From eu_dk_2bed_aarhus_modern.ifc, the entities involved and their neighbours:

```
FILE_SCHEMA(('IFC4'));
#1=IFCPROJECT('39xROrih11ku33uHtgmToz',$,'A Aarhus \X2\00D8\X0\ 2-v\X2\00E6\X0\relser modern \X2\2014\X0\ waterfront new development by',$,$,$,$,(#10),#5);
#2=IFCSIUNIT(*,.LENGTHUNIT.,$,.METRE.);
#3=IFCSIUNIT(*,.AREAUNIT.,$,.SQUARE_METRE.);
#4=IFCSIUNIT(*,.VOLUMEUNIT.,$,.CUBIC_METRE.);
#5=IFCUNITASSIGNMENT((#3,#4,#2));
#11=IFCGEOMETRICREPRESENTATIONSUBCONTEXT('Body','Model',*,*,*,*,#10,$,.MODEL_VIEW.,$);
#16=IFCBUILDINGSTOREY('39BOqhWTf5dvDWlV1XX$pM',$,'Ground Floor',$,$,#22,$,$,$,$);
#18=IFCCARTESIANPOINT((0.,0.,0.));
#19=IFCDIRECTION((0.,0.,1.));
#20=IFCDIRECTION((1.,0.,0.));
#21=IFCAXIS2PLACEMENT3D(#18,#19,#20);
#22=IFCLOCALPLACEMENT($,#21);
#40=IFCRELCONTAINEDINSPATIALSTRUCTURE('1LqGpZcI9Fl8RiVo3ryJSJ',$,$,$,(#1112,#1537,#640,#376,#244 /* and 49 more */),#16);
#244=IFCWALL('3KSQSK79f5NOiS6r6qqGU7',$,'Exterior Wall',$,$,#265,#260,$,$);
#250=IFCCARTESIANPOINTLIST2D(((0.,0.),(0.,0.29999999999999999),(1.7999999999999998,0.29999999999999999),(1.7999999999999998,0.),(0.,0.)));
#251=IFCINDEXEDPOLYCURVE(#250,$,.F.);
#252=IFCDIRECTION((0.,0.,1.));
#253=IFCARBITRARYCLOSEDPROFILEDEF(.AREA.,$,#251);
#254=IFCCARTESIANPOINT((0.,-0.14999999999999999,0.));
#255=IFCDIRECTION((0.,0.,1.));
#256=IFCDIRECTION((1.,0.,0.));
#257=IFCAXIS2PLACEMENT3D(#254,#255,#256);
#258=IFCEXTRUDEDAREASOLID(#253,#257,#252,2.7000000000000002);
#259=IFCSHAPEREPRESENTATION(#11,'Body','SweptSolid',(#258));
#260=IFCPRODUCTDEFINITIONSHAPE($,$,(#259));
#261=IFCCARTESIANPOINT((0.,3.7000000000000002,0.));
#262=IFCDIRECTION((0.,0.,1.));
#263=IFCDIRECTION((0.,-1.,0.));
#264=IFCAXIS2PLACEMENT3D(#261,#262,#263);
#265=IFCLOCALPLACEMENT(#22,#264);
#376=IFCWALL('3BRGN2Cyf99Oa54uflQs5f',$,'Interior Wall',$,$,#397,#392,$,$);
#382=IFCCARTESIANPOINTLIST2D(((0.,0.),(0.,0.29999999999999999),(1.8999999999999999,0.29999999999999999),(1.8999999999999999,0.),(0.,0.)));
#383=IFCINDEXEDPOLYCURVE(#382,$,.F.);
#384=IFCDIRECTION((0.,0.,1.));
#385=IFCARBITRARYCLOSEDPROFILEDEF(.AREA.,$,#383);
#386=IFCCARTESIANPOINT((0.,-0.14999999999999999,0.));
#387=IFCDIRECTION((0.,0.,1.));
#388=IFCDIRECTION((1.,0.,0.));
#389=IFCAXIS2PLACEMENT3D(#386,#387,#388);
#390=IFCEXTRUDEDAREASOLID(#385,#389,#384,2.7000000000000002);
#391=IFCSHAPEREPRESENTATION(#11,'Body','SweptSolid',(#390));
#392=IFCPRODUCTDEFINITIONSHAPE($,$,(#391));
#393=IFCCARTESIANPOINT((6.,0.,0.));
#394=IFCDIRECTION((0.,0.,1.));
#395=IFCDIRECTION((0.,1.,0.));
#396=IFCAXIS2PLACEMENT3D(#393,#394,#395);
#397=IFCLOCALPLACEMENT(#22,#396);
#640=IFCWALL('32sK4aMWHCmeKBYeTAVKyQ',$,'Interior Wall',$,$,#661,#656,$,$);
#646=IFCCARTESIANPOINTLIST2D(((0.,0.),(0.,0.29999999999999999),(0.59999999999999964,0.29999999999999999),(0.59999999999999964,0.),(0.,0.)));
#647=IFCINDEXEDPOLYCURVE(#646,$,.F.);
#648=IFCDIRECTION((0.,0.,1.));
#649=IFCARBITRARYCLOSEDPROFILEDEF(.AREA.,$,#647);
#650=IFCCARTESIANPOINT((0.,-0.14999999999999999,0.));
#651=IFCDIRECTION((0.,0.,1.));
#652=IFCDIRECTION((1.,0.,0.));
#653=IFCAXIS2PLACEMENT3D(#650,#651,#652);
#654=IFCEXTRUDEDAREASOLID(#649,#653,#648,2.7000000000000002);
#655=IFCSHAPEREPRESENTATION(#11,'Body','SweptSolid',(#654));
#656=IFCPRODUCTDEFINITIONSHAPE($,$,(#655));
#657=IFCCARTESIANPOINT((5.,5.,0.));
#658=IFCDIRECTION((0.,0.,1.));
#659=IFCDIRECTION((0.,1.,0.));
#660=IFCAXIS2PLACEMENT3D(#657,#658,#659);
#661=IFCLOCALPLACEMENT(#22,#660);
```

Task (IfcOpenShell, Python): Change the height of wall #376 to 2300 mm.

```python
import ifcopenshell
import ifcopenshell.geom
import ifcopenshell.util.representation
import ifcopenshell.util.shape
import ifcopenshell.util.unit

model = ifcopenshell.open("eu_dk_2bed_aarhus_modern.ifc")
unit_scale = ifcopenshell.util.unit.calculate_unit_scale(model)
settings = ifcopenshell.geom.settings()


def volume(element):
    """Net volume in cubic metres, openings subtracted."""
    shape = ifcopenshell.geom.create_shape(settings, element)
    return ifcopenshell.util.shape.get_volume(shape.geometry)


wall = model.by_id(376)
before = volume(wall)

body = ifcopenshell.util.representation.get_representation(wall, "Model", "Body")
solid = body.Items[0]
old_height = solid.Depth
solid.Depth = 2.3 / unit_scale
after = volume(wall)

print(f"height {old_height:g} -> {solid.Depth:g}, volume {before:.3f} -> {after:.3f} m3")

model.write("eu_dk_2bed_aarhus_modern_v2.ifc")
```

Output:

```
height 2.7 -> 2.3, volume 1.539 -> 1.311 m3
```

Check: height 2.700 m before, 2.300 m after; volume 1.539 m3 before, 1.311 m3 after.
